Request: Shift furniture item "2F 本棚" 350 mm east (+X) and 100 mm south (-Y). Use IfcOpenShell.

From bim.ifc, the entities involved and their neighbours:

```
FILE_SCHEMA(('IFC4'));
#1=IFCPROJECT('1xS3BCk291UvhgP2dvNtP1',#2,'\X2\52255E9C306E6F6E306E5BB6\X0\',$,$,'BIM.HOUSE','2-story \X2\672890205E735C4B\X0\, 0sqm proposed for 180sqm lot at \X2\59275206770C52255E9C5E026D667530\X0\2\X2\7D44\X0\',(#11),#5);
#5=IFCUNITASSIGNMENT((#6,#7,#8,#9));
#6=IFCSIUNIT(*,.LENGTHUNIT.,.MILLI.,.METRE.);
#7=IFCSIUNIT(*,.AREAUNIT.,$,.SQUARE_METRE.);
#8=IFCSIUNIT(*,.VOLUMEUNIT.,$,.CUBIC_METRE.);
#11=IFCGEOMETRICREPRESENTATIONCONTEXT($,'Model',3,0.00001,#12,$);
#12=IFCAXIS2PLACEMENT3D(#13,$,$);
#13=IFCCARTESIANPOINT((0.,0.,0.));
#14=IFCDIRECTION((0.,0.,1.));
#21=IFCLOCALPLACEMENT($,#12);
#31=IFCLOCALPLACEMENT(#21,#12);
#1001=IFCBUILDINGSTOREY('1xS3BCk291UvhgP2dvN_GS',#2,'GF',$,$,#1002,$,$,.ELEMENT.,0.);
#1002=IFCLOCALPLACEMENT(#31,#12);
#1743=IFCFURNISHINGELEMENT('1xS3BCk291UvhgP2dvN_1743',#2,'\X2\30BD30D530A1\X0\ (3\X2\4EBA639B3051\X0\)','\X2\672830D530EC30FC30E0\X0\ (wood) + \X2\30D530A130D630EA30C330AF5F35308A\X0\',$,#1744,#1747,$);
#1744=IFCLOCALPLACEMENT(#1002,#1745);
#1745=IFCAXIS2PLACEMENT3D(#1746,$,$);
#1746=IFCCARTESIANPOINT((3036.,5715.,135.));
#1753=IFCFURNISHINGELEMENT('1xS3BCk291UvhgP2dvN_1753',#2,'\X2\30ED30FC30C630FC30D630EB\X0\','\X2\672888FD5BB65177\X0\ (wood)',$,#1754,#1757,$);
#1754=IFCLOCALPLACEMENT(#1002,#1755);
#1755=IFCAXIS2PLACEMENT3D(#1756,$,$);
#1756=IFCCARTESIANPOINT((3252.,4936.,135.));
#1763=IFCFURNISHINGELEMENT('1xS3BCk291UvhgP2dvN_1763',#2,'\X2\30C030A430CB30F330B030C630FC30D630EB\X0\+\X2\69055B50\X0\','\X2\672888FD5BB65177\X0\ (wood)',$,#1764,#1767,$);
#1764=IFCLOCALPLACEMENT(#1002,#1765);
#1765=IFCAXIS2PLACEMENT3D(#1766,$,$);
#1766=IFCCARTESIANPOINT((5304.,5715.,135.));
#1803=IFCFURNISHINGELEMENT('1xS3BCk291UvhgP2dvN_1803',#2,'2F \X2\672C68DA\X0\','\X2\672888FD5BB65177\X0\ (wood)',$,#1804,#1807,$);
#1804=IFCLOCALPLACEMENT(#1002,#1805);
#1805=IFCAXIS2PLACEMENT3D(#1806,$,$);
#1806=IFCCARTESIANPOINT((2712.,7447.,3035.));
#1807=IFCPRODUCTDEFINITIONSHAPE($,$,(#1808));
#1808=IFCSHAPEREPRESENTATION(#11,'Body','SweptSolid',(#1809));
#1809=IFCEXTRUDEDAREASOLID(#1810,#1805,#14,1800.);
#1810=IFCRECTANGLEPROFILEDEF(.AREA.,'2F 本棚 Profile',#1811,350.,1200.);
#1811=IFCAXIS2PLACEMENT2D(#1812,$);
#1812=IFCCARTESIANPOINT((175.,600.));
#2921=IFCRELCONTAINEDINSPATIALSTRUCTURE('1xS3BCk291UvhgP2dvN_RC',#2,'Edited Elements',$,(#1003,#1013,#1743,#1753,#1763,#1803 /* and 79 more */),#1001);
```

```python
import ifcopenshell
import ifcopenshell.api.geometry
import ifcopenshell.util.placement
import ifcopenshell.util.unit

model = ifcopenshell.open("bim.ifc")
unit_scale = ifcopenshell.util.unit.calculate_unit_scale(model)

item = model.by_guid("1xS3BCk291UvhgP2dvN_1803")
matrix = ifcopenshell.util.placement.get_local_placement(item.ObjectPlacement)
matrix[0, 3] += 0.35 / unit_scale
matrix[1, 3] -= 0.1 / unit_scale
ifcopenshell.api.geometry.edit_object_placement(model, product=item, matrix=matrix, is_si=False)

print(ifcopenshell.util.placement.get_local_placement(item.ObjectPlacement).round(3) + 0.0)

model.write("bim_updated.ifc")
```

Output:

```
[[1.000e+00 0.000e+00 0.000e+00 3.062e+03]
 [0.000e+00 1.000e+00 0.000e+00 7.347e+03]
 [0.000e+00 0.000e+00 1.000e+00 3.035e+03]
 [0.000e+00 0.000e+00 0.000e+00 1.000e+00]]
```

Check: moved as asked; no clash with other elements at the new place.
